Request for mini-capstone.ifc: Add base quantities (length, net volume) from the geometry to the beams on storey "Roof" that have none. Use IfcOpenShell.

First a look at what the model holds.

```python
import ifcopenshell
import ifcopenshell.util.element
import ifcopenshell.util.unit

model = ifcopenshell.open("mini-capstone.ifc")
print(model.schema)
for unit_type in ("LENGTHUNIT", "AREAUNIT", "VOLUMEUNIT"):
    print(unit_type, ifcopenshell.util.unit.calculate_unit_scale(model, unit_type))
storey = next(s for s in model.by_type("IfcBuildingStorey") if s.Name == "Roof")
beams = [e for e in ifcopenshell.util.element.get_decomposition(storey) if e.is_a("IfcBeam")]
for e in sorted(beams, key=lambda e: e.id()):
    print(e.id(), e.is_a(), e.Name, list(ifcopenshell.util.element.get_psets(e, qtos_only=True)), sep=" | ")
```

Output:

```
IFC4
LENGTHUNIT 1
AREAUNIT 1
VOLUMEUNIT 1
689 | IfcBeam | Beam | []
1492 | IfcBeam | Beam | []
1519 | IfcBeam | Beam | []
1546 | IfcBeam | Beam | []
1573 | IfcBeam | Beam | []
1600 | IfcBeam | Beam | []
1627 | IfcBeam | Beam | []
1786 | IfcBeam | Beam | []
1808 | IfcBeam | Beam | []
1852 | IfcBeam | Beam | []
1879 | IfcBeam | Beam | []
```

```python
import ifcopenshell
import ifcopenshell.api.pset
import ifcopenshell.geom
import ifcopenshell.util.element
import ifcopenshell.util.shape
import ifcopenshell.util.unit

model = ifcopenshell.open("mini-capstone.ifc")
unit_scale = ifcopenshell.util.unit.calculate_unit_scale(model)
volume_scale = ifcopenshell.util.unit.calculate_unit_scale(model, "VOLUMEUNIT")
settings = ifcopenshell.geom.settings()

storey = next(s for s in model.by_type("IfcBuildingStorey") if s.Name == "Roof")
beams = [e for e in ifcopenshell.util.element.get_decomposition(storey) if e.is_a("IfcBeam")]

for e in sorted(beams, key=lambda e: e.id()):
    if ifcopenshell.util.element.get_psets(e, qtos_only=True, should_inherit=False):
        continue
    # Geometry comes back in metres, in the element's own axes.
    shape = ifcopenshell.geom.create_shape(settings, e)
    values = {
        "Length": ifcopenshell.util.shape.get_max_xyz(shape.geometry) / unit_scale,
        "NetVolume": ifcopenshell.util.shape.get_volume(shape.geometry) / volume_scale,
    }
    qto = ifcopenshell.api.pset.add_qto(model, product=e, name="Qto_BeamBaseQuantities")
    ifcopenshell.api.pset.edit_qto(model, qto=qto, properties=values)
    print(e.id(), {k: round(v, 3) for k, v in values.items()})

model.write("mini-capstone_rev.ifc")
```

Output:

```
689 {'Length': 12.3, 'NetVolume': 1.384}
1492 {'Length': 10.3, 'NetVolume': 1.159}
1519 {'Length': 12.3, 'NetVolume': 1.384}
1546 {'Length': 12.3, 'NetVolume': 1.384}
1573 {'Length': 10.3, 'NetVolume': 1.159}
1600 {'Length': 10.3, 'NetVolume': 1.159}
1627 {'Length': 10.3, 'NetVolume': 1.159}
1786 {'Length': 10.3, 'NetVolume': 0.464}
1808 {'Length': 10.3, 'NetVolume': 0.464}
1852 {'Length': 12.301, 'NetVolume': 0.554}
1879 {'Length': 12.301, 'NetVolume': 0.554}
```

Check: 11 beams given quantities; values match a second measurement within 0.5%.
